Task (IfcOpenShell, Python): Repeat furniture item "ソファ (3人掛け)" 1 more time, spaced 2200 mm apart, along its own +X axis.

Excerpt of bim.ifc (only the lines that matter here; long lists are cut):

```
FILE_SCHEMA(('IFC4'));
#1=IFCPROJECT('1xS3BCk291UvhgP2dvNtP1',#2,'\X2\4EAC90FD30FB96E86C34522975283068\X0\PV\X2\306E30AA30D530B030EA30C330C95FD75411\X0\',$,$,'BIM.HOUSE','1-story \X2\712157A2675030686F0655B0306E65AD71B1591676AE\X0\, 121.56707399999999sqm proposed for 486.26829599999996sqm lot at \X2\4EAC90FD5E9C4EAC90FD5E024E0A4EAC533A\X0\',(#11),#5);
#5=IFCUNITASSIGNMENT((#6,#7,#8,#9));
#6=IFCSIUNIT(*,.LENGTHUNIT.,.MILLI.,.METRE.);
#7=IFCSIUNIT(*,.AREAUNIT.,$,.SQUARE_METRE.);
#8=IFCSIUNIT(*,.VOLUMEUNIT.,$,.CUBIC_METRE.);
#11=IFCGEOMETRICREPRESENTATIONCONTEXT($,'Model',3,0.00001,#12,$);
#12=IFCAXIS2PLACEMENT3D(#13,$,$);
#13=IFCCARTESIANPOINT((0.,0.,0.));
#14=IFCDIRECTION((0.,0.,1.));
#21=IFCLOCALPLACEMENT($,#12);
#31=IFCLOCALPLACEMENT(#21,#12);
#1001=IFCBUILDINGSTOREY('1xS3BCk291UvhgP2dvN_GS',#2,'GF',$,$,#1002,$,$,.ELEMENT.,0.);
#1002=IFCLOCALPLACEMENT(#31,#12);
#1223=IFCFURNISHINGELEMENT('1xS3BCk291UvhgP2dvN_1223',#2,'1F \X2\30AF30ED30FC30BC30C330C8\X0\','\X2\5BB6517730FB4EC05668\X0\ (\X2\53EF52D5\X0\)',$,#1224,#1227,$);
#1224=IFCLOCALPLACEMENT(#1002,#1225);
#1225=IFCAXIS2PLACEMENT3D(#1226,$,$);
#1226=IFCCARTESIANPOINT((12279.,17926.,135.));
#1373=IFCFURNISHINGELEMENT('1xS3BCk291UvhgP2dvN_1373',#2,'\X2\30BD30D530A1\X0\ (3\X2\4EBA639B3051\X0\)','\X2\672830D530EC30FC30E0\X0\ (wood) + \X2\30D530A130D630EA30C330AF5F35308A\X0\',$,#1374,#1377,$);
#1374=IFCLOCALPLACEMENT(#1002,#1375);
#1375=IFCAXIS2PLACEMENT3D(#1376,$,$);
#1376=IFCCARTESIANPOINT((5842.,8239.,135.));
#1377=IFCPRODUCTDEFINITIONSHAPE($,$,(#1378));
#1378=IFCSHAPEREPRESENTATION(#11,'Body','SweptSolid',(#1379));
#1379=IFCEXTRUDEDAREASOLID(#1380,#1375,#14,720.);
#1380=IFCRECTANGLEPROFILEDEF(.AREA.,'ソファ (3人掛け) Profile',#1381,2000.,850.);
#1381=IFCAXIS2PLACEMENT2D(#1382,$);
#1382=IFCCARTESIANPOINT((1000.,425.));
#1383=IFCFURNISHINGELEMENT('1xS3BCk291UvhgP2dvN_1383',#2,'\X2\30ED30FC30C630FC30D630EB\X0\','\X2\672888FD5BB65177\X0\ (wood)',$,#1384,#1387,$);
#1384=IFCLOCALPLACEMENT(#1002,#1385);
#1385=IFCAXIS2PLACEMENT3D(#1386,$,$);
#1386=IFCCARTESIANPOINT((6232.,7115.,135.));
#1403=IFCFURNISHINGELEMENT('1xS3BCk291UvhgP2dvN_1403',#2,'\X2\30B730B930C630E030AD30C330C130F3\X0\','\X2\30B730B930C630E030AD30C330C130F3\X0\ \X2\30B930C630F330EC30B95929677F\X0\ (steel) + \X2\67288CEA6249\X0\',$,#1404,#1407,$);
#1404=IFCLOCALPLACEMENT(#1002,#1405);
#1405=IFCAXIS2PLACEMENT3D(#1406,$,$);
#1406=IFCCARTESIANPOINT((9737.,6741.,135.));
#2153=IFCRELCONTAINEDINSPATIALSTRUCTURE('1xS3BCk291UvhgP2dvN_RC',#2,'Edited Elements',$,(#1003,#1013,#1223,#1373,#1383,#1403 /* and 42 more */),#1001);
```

```python
import ifcopenshell
import ifcopenshell.api.geometry
import ifcopenshell.api.root
import ifcopenshell.util.element
import ifcopenshell.util.placement

model = ifcopenshell.open("bim.ifc")


def reuse_history(source, copy):
    """copy_class also copies each property set's owner history, people and application; keep the originals."""
    for rel in copy.IsDefinedBy:
        if rel.is_a("IfcRelDefinesByProperties") and (history := rel.RelatingPropertyDefinition.OwnerHistory):
            rel.RelatingPropertyDefinition.OwnerHistory = source.OwnerHistory
            ifcopenshell.util.element.remove_deep2(model, history)


source = model.by_guid("1xS3BCk291UvhgP2dvN_1373")
base = ifcopenshell.util.placement.get_local_placement(source.ObjectPlacement)
step = base[:3, 0] * 2200.0

for i in range(1, 2):
    copy = ifcopenshell.api.root.copy_class(model, product=source)
    copy.Representation = ifcopenshell.util.element.copy_deep(
        model, source.Representation, exclude=["IfcGeometricRepresentationContext", "IfcRepresentationMap"]
    )
    reuse_history(source, copy)
    matrix = base.copy()
    matrix[:3, 3] += i * step
    print("added at", matrix[:3, 3].round(3) + 0.0)
    ifcopenshell.api.geometry.edit_object_placement(model, product=copy, matrix=matrix, is_si=False)

model.write("bim_v2.ifc")
```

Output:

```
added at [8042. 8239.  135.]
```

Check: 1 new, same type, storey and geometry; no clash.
